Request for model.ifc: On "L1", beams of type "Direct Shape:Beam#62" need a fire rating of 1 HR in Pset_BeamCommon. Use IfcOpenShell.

First a look at what the model holds.

```python
import ifcopenshell
import ifcopenshell.util.element

model = ifcopenshell.open("model.ifc")
print(model.schema)
storey = next(s for s in model.by_type("IfcBuildingStorey") if s.Name == "L1")
beams = [e for e in ifcopenshell.util.element.get_decomposition(storey) if e.is_a("IfcBeam")]
seen = {}
for e in beams:
    element_type = ifcopenshell.util.element.get_type(e)
    key = (element_type.Name if element_type != e and element_type else None, ifcopenshell.util.element.get_pset(e, "Pset_BeamCommon", "FireRating"))
    seen[key] = seen.get(key, 0) + 1
for (name, value), count in sorted(seen.items(), key=str):
    print(count, "x", name, "|", value)
```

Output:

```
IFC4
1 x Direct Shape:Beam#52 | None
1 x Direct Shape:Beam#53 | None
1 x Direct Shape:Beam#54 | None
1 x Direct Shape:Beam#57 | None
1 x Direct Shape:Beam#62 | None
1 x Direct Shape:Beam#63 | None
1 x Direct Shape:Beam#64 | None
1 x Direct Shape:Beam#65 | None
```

```python
import ifcopenshell
import ifcopenshell.api.pset
import ifcopenshell.util.element

model = ifcopenshell.open("model.ifc")

storey = next(s for s in model.by_type("IfcBuildingStorey") if s.Name == "L1")
beams = [e for e in ifcopenshell.util.element.get_decomposition(storey) if e.is_a("IfcBeam")]

count = 0
for e in beams:
    element_type = ifcopenshell.util.element.get_type(e)
    if element_type in (None, e) or element_type.Name != "Direct Shape:Beam#62":
        continue
    # add_pset returns the element's existing set when there is one.
    pset = ifcopenshell.api.pset.add_pset(model, product=e, name="Pset_BeamCommon")
    ifcopenshell.api.pset.edit_pset(model, pset=pset, properties={"FireRating": "1 HR"})
    count += 1

print(count, "beams updated")

model.write("model_rev.ifc")
```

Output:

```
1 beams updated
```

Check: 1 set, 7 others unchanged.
